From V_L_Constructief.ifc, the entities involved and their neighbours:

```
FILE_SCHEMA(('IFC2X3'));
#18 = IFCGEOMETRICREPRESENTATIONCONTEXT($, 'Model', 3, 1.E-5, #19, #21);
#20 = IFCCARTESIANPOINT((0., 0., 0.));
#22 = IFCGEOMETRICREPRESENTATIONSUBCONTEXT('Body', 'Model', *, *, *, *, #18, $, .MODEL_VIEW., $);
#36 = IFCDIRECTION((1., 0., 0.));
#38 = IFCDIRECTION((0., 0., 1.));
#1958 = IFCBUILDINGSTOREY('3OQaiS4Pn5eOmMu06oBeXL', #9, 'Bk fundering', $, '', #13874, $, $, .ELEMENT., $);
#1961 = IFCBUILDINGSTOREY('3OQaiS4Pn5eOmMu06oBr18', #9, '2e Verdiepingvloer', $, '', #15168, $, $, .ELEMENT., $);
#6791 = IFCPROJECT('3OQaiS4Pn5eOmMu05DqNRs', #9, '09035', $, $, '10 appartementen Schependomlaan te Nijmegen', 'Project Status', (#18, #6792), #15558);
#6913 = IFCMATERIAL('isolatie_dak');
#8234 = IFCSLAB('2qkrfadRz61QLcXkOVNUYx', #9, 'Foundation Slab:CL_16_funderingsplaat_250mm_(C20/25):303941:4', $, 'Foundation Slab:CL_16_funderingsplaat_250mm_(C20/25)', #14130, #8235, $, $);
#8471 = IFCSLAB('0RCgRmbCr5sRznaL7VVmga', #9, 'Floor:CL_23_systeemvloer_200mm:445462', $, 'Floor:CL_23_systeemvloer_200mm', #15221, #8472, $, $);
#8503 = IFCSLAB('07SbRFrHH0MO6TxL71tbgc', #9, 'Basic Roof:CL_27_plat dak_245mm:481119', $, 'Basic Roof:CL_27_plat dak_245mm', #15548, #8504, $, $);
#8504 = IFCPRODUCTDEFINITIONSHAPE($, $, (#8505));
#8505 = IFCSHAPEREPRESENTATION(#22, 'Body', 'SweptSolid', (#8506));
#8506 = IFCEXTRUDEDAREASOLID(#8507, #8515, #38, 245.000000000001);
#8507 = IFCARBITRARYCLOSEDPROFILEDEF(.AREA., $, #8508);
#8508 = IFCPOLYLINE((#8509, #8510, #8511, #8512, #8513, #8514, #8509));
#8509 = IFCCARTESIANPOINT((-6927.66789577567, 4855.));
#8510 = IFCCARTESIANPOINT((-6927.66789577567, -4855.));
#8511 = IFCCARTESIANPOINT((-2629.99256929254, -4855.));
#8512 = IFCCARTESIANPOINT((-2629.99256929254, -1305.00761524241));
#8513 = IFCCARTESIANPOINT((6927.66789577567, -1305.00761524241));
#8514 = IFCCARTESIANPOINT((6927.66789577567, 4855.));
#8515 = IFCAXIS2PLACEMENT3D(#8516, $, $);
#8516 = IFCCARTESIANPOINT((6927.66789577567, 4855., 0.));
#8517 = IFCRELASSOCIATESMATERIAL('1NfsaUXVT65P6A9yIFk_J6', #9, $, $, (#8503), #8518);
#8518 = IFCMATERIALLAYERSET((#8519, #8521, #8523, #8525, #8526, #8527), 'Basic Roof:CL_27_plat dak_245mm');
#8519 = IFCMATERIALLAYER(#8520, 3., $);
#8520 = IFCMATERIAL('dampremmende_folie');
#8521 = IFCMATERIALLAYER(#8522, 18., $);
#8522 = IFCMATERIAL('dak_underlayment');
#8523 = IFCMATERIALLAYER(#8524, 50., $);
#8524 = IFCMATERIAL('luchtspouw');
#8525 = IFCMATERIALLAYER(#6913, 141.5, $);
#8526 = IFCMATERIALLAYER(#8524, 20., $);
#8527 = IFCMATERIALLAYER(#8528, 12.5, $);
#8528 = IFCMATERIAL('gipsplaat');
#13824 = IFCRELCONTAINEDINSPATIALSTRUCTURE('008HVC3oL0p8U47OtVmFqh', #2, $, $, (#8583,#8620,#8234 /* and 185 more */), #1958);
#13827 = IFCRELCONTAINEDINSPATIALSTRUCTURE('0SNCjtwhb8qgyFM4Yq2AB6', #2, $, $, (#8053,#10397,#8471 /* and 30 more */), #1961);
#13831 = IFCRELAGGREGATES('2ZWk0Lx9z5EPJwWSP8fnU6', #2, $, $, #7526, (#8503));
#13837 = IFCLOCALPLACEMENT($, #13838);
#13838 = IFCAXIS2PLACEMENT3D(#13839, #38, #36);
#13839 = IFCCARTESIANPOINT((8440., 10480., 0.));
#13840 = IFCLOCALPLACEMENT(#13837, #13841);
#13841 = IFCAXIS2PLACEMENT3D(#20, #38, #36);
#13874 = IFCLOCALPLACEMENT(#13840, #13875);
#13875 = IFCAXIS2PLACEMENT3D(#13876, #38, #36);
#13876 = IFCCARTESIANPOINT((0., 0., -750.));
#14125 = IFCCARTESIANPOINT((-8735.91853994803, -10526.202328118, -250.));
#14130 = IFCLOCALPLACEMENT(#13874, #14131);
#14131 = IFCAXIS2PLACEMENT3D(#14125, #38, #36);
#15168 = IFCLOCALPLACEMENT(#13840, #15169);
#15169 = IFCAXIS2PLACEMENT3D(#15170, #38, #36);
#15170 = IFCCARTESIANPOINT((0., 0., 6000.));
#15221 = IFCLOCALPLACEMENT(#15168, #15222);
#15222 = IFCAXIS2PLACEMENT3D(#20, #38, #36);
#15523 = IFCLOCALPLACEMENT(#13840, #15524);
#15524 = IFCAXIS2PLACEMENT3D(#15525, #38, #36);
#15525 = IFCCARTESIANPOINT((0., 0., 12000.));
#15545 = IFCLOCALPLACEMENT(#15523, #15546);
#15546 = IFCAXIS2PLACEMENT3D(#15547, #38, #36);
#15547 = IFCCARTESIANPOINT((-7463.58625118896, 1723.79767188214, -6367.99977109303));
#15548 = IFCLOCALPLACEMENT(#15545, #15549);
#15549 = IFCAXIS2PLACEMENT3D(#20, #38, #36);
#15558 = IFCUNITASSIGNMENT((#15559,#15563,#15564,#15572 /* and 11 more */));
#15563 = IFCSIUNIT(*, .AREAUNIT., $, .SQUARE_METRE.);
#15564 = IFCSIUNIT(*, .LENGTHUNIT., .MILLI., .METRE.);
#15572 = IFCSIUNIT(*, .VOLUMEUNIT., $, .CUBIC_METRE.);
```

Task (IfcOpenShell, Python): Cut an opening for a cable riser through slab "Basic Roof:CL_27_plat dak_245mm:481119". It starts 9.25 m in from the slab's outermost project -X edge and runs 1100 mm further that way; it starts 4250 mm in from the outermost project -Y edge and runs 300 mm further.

```python
import numpy as np
import ifcopenshell
import ifcopenshell.api.feature
import ifcopenshell.api.geometry
import ifcopenshell.api.root
import ifcopenshell.geom
import ifcopenshell.util.placement
import ifcopenshell.util.representation
import ifcopenshell.util.shape
import ifcopenshell.util.unit

model = ifcopenshell.open("V_L_Constructief.ifc")
unit_scale = ifcopenshell.util.unit.calculate_unit_scale(model)
settings = ifcopenshell.geom.settings()


def volume(element):
    """Net volume in cubic metres, openings subtracted."""
    shape = ifcopenshell.geom.create_shape(settings, element)
    return ifcopenshell.util.shape.get_volume(shape.geometry)


slab = model.by_guid("07SbRFrHH0MO6TxL71tbgc")
before = volume(slab)

# Extent in the slab's own axes, in metres. The edges named are its -X and -Y sides.
slab_shape = ifcopenshell.geom.create_shape(settings, slab)
vertices = ifcopenshell.util.shape.get_vertices(slab_shape.geometry)
x_min, y_min, bottom = vertices.min(axis=0)
top = vertices[:, 2].max()

opening = ifcopenshell.api.root.create_entity(model, ifc_class="IfcOpeningElement", name="Cable riser opening")
context = ifcopenshell.util.representation.get_context(model, "Model", "Body", "MODEL_VIEW")
width, depth = 1.1, 0.3
outline = [(0.0, 0.0), (width, 0.0), (width, depth), (0.0, depth), (0.0, 0.0)]
# Overshoot both faces by 50 mm so the cut is clean.
shape = ifcopenshell.api.geometry.add_slab_representation(
    model, context=context, depth=top - bottom + 0.1, polyline=outline
)
ifcopenshell.api.geometry.assign_representation(model, product=opening, representation=shape)

matrix = ifcopenshell.util.placement.get_local_placement(slab.ObjectPlacement)
matrix[:, 3] = matrix @ np.append(np.array([x_min + 9.25, y_min + 4.25, bottom - 0.05]) / unit_scale, 1.0)
ifcopenshell.api.geometry.edit_object_placement(model, product=opening, matrix=matrix, is_si=False)
ifcopenshell.api.feature.add_feature(model, feature=opening, element=slab)

after = volume(slab)

print(f"slab volume {before:.3f} -> {after:.3f} m3")

model.write("V_L_Constructief_rev.ifc")
```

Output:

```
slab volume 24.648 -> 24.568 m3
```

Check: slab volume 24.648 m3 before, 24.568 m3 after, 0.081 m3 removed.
